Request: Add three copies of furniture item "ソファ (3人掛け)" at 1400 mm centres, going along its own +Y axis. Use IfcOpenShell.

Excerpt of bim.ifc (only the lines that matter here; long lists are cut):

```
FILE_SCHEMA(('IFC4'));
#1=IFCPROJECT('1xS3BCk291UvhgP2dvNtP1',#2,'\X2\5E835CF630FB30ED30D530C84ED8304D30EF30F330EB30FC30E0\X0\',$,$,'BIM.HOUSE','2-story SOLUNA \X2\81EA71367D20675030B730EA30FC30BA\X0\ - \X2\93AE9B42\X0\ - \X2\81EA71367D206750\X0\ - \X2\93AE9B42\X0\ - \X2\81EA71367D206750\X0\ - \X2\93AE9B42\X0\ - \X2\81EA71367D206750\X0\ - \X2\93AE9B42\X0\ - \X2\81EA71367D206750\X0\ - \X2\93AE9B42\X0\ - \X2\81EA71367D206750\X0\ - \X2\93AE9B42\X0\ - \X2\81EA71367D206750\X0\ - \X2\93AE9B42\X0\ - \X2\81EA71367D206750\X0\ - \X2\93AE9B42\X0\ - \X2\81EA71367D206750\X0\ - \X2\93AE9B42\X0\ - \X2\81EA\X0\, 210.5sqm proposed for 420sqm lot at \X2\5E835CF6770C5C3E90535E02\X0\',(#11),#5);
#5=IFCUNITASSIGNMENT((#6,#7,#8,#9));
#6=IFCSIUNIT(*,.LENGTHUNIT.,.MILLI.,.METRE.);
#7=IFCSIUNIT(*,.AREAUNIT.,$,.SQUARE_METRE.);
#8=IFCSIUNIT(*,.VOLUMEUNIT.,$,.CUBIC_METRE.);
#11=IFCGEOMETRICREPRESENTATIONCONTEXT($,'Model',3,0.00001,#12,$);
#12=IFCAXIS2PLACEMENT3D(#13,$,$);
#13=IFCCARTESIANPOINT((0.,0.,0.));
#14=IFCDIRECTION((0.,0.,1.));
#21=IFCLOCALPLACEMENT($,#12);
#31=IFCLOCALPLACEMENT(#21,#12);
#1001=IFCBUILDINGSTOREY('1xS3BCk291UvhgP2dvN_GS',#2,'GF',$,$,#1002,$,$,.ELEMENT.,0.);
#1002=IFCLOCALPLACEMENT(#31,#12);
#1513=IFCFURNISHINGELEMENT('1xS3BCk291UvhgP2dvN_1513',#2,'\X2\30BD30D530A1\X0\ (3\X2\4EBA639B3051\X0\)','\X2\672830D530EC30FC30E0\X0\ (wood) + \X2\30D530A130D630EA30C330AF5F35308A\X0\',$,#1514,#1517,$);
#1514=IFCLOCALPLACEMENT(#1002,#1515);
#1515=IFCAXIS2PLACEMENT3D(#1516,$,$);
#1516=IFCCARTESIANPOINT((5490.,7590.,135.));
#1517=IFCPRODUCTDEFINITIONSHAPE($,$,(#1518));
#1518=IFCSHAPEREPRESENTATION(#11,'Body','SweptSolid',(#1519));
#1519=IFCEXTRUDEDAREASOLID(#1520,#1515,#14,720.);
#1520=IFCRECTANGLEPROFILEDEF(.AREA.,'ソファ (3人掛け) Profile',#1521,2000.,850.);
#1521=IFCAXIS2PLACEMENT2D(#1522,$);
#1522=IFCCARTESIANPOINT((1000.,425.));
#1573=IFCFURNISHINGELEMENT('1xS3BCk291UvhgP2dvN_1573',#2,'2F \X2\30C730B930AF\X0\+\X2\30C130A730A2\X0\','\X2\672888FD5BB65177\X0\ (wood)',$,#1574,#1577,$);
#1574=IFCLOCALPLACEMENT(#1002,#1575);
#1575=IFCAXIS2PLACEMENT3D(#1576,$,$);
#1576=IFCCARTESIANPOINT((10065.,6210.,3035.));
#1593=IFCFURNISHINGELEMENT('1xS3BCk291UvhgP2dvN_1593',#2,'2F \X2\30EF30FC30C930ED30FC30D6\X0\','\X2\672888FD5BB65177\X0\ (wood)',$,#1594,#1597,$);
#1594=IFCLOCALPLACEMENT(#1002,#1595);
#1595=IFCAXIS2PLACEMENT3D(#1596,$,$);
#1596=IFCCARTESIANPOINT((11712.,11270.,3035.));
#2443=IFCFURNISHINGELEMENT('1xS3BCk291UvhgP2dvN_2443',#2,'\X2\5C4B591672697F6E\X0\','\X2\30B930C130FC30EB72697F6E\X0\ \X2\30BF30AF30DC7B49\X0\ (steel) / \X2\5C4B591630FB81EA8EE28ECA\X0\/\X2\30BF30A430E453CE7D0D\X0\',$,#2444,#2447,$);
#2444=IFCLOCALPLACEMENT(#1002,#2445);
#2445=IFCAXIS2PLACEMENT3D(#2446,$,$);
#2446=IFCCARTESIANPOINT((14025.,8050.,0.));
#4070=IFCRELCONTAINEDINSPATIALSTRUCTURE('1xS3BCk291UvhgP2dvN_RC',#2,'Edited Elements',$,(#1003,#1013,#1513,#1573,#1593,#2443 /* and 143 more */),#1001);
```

```python
import ifcopenshell
import ifcopenshell.api.geometry
import ifcopenshell.api.root
import ifcopenshell.util.element
import ifcopenshell.util.placement
import ifcopenshell.util.unit

model = ifcopenshell.open("bim.ifc")
unit_scale = ifcopenshell.util.unit.calculate_unit_scale(model)


def reuse_history(source, copy):
    """copy_class also copies each property set's owner history, people and application; keep the originals."""
    for rel in copy.IsDefinedBy:
        if rel.is_a("IfcRelDefinesByProperties") and (history := rel.RelatingPropertyDefinition.OwnerHistory):
            rel.RelatingPropertyDefinition.OwnerHistory = source.OwnerHistory
            ifcopenshell.util.element.remove_deep2(model, history)


source = model.by_guid("1xS3BCk291UvhgP2dvN_1513")
base = ifcopenshell.util.placement.get_local_placement(source.ObjectPlacement)
step = base[:3, 1] * 1.4 / unit_scale

for i in range(1, 4):
    copy = ifcopenshell.api.root.copy_class(model, product=source)
    copy.Representation = ifcopenshell.util.element.copy_deep(
        model, source.Representation, exclude=["IfcGeometricRepresentationContext", "IfcRepresentationMap"]
    )
    reuse_history(source, copy)
    matrix = base.copy()
    matrix[:3, 3] += i * step
    print("added at", matrix[:3, 3].round(3) + 0.0)
    ifcopenshell.api.geometry.edit_object_placement(model, product=copy, matrix=matrix, is_si=False)

model.write("bim_updated.ifc")
```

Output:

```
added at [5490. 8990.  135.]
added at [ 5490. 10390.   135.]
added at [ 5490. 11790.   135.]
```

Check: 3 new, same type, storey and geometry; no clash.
